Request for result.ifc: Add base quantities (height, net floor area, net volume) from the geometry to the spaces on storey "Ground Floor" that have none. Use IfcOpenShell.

First a look at what the model holds.

```python
import ifcopenshell
import ifcopenshell.util.element
import ifcopenshell.util.unit

model = ifcopenshell.open("result.ifc")
print(model.schema)
for unit_type in ("LENGTHUNIT", "AREAUNIT", "VOLUMEUNIT"):
    print(unit_type, ifcopenshell.util.unit.calculate_unit_scale(model, unit_type))
storey = next(s for s in model.by_type("IfcBuildingStorey") if s.Name == "Ground Floor")
spaces = [e for e in ifcopenshell.util.element.get_decomposition(storey) if e.is_a("IfcSpace")]
for e in sorted(spaces, key=lambda e: e.id()):
    print(e.id(), e.is_a(), e.Name, list(ifcopenshell.util.element.get_psets(e, qtos_only=True)), sep=" | ")
```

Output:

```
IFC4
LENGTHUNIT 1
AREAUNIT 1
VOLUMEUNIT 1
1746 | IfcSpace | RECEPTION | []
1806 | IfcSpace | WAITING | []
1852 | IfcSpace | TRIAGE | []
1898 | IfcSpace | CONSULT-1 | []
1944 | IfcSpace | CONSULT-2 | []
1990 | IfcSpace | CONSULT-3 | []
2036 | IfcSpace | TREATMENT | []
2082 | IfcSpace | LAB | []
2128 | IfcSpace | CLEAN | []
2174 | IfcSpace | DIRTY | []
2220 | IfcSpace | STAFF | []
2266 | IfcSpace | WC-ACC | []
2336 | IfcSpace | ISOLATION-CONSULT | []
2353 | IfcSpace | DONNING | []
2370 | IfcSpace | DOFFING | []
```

```python
import ifcopenshell
import ifcopenshell.api.pset
import ifcopenshell.geom
import ifcopenshell.util.element
import ifcopenshell.util.shape
import ifcopenshell.util.unit

model = ifcopenshell.open("result.ifc")
unit_scale = ifcopenshell.util.unit.calculate_unit_scale(model)
area_scale = ifcopenshell.util.unit.calculate_unit_scale(model, "AREAUNIT")
volume_scale = ifcopenshell.util.unit.calculate_unit_scale(model, "VOLUMEUNIT")
settings = ifcopenshell.geom.settings()

storey = next(s for s in model.by_type("IfcBuildingStorey") if s.Name == "Ground Floor")
spaces = [e for e in ifcopenshell.util.element.get_decomposition(storey) if e.is_a("IfcSpace")]

for e in sorted(spaces, key=lambda e: e.id()):
    if ifcopenshell.util.element.get_psets(e, qtos_only=True, should_inherit=False):
        continue
    # Geometry comes back in metres, in the element's own axes.
    shape = ifcopenshell.geom.create_shape(settings, e)
    values = {
        "Height": ifcopenshell.util.shape.get_z(shape.geometry) / unit_scale,
        "NetFloorArea": ifcopenshell.util.shape.get_footprint_area(shape.geometry) / area_scale,
        "NetVolume": ifcopenshell.util.shape.get_volume(shape.geometry) / volume_scale,
    }
    qto = ifcopenshell.api.pset.add_qto(model, product=e, name="Qto_SpaceBaseQuantities")
    ifcopenshell.api.pset.edit_qto(model, qto=qto, properties=values)
    print(e.id(), {k: round(v, 3) for k, v in values.items()})

model.write("result-out.ifc")
```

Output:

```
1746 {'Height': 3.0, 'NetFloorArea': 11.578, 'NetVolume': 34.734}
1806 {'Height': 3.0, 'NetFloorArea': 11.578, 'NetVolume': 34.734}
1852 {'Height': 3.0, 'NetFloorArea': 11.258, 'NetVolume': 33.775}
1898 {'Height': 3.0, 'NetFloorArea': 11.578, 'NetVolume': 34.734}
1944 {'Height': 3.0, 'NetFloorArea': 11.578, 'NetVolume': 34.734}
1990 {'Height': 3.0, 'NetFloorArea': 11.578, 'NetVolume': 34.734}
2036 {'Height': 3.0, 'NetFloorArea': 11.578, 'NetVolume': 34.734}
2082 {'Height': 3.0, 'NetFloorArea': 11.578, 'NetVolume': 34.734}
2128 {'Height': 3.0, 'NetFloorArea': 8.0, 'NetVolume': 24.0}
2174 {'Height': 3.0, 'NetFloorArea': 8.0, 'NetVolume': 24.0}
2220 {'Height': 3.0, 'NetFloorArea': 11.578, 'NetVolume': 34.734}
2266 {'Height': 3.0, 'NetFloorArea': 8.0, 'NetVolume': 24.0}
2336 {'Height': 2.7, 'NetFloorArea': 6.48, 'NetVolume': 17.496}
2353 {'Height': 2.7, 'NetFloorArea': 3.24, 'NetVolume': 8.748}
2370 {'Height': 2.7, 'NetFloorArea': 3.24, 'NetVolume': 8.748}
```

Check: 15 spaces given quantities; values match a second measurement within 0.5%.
